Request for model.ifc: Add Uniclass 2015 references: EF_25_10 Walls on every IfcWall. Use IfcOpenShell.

First a look at what the model holds.

```python
import ifcopenshell

model = ifcopenshell.open("model.ifc")
print(model.schema)
print("classifications:", [c.Name for c in model.by_type("IfcClassification")])
for ifc_class in ("IfcDoor", "IfcRoof", "IfcStair", "IfcWall", "IfcWindow"):
    print(ifc_class, len(model.by_type(ifc_class)))
```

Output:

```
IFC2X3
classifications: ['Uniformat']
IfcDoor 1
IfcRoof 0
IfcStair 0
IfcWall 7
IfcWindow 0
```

```python
import ifcopenshell
import ifcopenshell.api.classification

model = ifcopenshell.open("model.ifc")

# IFC2X3 requires Source and Edition and has no link from the project to the system.
system = model.create_entity("IfcClassification", Source="NBS", Edition="2015", Name="Uniclass 2015")

codes = {
    "IfcWall": ("EF_25_10", "Walls"),
}
for ifc_class, (code, name) in codes.items():
    products = model.by_type(ifc_class)
    ifcopenshell.api.classification.add_reference(
        model, products=products, classification=system, identification=code, name=name
    )
    print(code, len(products))

model.write("model-out.ifc")
```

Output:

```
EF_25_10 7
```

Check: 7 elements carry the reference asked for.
